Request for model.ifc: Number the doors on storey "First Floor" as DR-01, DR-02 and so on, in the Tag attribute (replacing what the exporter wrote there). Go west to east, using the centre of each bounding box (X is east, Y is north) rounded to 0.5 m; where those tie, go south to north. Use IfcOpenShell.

First a look at what the model holds.

```python
import ifcopenshell
import ifcopenshell.util.element
import ifcopenshell.util.placement

model = ifcopenshell.open("model.ifc")
print(model.schema)
storey = next(s for s in model.by_type("IfcBuildingStorey") if s.Name == "First Floor")
doors = [e for e in ifcopenshell.util.element.get_decomposition(storey) if e.is_a("IfcDoor")]
for e in sorted(doors, key=lambda e: e.id()):
    origin = ifcopenshell.util.placement.get_local_placement(e.ObjectPlacement)[:3, 3]
    print(e.id(), e.Tag, e.Name, origin.round(2) + 0.0, sep=" | ")
```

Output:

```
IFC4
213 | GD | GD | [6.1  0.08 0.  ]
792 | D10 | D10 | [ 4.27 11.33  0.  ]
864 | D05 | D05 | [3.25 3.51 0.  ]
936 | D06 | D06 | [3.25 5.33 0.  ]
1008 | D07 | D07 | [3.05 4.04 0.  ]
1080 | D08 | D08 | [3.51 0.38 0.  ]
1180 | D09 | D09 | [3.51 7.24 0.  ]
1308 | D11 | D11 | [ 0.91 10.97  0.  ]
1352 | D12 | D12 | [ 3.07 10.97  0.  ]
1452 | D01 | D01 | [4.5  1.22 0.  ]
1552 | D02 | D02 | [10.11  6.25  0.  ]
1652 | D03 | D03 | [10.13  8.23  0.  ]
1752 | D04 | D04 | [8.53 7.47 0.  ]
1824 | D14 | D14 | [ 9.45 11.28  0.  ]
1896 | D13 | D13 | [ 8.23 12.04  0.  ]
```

```python
import ifcopenshell
import ifcopenshell.geom
import ifcopenshell.util.element
import ifcopenshell.util.shape

model = ifcopenshell.open("model.ifc")
settings = ifcopenshell.geom.settings()
settings.set("use-world-coords", True)


def centre(element):
    shape = ifcopenshell.geom.create_shape(settings, element)
    return ifcopenshell.util.shape.get_bbox_centroid(shape.geometry)


storey = next(s for s in model.by_type("IfcBuildingStorey") if s.Name == "First Floor")
doors = [e for e in ifcopenshell.util.element.get_decomposition(storey) if e.is_a("IfcDoor")]

# Insertion points can sit at a corner or the storey origin, so sort by the geometry (in metres).
centres = {e: centre(e) for e in doors}
doors.sort(key=lambda e: (round(centres[e][0] / 0.5), centres[e][1]))

for i, e in enumerate(doors, start=1):
    number = f"DR-{i:02d}"
    e.Tag = number
    print(e.id(), number)

model.write("model_rev.ifc")
```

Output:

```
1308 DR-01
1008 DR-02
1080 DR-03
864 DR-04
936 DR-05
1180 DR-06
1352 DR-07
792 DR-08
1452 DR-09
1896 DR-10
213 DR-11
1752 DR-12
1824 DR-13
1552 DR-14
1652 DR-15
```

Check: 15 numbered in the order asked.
